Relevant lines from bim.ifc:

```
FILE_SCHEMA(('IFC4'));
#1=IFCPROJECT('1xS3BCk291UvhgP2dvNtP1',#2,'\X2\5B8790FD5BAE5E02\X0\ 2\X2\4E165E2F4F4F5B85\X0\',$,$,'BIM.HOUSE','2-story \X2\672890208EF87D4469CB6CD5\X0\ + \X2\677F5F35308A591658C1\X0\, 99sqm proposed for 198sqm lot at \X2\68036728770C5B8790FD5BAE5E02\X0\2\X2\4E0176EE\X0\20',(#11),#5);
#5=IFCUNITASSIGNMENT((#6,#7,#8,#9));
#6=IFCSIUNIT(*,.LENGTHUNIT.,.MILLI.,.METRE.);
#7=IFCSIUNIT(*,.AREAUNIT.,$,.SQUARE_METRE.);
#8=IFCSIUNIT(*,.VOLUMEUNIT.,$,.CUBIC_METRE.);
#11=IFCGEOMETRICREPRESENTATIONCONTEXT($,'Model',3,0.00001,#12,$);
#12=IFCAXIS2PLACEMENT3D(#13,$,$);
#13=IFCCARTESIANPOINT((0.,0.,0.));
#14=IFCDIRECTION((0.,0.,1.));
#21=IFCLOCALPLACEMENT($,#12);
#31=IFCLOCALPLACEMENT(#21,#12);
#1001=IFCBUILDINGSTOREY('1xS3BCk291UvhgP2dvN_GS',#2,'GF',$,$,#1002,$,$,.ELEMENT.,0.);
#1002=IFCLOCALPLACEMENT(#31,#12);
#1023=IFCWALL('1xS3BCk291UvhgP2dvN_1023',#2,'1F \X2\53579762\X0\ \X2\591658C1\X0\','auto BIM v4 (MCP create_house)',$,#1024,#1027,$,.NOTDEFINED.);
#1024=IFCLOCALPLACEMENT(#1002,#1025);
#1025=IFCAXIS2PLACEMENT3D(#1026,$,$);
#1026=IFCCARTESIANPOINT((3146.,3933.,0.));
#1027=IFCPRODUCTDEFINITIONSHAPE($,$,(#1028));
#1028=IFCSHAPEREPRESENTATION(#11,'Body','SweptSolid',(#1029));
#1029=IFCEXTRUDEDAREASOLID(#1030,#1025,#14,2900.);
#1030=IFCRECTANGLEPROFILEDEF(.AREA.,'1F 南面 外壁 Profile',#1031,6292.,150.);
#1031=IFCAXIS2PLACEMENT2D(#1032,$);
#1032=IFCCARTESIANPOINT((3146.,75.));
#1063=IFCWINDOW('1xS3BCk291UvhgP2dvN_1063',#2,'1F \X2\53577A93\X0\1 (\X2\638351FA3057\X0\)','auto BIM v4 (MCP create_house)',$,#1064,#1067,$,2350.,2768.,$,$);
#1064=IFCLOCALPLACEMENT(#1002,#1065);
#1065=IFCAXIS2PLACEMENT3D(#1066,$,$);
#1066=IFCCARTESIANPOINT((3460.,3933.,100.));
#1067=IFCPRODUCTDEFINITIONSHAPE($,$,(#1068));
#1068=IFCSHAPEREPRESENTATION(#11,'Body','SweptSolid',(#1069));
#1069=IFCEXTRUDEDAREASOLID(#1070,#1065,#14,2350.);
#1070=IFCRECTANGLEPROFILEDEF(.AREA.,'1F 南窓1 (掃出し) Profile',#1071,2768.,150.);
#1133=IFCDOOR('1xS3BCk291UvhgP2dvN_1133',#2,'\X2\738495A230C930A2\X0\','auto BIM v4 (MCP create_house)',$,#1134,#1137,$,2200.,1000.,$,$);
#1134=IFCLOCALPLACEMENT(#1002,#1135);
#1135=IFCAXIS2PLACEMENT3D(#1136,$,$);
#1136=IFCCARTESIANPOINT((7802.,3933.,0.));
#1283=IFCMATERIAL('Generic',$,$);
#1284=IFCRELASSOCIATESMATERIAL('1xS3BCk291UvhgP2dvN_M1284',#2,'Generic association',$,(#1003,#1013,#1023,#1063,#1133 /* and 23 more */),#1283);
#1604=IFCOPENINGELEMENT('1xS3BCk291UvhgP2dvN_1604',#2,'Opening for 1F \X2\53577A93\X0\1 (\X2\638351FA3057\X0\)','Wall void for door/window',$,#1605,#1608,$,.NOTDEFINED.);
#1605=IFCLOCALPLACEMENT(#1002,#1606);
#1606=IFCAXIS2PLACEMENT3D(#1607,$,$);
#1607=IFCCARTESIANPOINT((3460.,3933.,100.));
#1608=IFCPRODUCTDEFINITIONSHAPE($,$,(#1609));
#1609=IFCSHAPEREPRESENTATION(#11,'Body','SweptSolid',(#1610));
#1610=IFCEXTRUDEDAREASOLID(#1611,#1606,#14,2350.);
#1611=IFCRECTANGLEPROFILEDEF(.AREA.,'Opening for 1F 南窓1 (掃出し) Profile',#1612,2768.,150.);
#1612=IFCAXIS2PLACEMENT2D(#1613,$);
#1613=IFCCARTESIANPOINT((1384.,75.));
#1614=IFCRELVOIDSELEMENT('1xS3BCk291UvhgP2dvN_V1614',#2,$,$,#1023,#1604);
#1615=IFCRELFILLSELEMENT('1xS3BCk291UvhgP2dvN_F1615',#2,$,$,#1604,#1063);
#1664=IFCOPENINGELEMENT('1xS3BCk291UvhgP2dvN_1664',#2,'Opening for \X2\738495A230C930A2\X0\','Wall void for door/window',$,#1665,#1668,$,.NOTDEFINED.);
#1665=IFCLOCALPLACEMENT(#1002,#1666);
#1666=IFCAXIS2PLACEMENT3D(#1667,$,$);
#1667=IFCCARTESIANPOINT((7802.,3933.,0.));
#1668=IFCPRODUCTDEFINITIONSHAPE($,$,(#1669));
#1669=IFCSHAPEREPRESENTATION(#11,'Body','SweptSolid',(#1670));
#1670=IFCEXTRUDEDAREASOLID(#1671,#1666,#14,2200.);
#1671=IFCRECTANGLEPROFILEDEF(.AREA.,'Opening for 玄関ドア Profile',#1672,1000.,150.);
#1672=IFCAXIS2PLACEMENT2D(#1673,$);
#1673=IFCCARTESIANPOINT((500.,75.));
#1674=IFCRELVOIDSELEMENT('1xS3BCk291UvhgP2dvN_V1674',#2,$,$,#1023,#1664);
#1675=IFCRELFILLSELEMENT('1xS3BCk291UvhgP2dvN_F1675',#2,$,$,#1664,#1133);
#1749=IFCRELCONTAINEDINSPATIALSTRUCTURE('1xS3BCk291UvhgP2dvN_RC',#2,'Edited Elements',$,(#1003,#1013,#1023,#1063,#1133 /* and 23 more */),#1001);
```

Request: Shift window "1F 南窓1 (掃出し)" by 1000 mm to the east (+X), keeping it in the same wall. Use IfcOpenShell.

```python
import ifcopenshell
import ifcopenshell.api.geometry
import ifcopenshell.util.placement
import ifcopenshell.util.unit

model = ifcopenshell.open("bim.ifc")
unit_scale = ifcopenshell.util.unit.calculate_unit_scale(model)

window = model.by_guid("1xS3BCk291UvhgP2dvN_1063")
opening = window.FillsVoids[0].RelatingOpeningElement
wall = opening.VoidsElements[0].RelatingBuildingElement

wall_matrix = ifcopenshell.util.placement.get_local_placement(wall.ObjectPlacement)
shift = wall_matrix[:3, 0] * 1 / unit_scale
before = ifcopenshell.util.placement.get_local_placement(window.ObjectPlacement)[:3, 3].copy()

# The window is not placed relative to its opening, so move both.
for product in (opening, window):
    matrix = ifcopenshell.util.placement.get_local_placement(product.ObjectPlacement)
    matrix[:3, 3] += shift
    ifcopenshell.api.geometry.edit_object_placement(model, product=product, matrix=matrix, is_si=False)

after = ifcopenshell.util.placement.get_local_placement(window.ObjectPlacement)[:3, 3]
print("window moved by", (after - before).round(3) + 0.0)

model.write("bim-out.ifc")
```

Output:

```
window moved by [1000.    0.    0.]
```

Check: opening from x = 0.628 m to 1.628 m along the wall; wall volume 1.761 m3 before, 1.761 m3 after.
